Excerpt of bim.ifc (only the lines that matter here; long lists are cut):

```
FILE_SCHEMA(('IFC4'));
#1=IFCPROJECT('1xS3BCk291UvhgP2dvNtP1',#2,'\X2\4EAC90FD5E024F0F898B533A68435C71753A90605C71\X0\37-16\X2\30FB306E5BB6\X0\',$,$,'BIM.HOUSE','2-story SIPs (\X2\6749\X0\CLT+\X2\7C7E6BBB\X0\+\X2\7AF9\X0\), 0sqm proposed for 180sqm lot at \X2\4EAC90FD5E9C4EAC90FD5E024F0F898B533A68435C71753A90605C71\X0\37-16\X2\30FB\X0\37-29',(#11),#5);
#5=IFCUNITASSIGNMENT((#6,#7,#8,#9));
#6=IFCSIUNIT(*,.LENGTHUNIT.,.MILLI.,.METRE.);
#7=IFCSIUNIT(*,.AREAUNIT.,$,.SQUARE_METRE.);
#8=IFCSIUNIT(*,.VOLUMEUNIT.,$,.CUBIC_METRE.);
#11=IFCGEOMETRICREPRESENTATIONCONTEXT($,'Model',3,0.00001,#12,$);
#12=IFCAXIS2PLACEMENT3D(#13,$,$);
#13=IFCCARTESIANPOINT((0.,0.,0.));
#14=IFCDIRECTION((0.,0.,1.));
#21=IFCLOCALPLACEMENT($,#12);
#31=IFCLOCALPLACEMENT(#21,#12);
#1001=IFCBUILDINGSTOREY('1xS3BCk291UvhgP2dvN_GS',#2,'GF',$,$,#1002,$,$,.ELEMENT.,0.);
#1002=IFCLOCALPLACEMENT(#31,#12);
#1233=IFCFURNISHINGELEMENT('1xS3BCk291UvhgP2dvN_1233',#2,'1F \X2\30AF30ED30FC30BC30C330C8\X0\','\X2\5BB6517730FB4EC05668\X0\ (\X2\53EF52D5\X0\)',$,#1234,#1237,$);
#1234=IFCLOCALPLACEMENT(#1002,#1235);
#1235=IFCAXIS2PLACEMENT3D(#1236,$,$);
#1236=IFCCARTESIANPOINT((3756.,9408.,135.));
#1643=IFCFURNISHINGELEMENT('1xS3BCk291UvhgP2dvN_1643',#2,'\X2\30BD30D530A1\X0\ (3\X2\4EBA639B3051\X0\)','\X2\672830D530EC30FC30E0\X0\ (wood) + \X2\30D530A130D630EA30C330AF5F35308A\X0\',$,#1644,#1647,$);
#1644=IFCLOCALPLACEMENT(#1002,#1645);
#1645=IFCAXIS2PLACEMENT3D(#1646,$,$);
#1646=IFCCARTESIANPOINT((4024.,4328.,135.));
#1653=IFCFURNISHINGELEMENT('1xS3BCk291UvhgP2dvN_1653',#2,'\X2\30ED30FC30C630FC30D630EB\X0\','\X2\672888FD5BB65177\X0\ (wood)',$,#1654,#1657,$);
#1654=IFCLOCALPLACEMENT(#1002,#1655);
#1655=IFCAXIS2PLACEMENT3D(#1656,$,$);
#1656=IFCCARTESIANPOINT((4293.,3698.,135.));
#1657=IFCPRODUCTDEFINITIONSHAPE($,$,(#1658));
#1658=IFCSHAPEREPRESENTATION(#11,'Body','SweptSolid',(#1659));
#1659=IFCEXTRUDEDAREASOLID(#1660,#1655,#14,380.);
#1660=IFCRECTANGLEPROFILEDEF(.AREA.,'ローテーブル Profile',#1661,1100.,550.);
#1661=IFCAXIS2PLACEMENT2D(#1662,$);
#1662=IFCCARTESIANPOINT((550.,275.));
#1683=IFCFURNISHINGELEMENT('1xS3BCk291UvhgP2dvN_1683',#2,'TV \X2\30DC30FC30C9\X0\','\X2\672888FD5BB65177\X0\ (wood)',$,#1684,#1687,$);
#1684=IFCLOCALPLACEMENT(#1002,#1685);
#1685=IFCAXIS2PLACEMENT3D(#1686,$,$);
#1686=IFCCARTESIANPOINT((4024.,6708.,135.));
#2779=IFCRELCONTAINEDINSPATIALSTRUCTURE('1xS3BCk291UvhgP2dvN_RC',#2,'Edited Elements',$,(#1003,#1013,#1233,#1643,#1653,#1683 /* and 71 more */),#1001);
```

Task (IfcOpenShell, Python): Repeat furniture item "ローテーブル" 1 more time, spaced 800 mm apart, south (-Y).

```python
import numpy as np
import ifcopenshell
import ifcopenshell.api.geometry
import ifcopenshell.api.root
import ifcopenshell.util.element
import ifcopenshell.util.placement

model = ifcopenshell.open("bim.ifc")


def reuse_history(source, copy):
    """copy_class also copies each property set's owner history, people and application; keep the originals."""
    for rel in copy.IsDefinedBy:
        if rel.is_a("IfcRelDefinesByProperties") and (history := rel.RelatingPropertyDefinition.OwnerHistory):
            rel.RelatingPropertyDefinition.OwnerHistory = source.OwnerHistory
            ifcopenshell.util.element.remove_deep2(model, history)


source = model.by_guid("1xS3BCk291UvhgP2dvN_1653")
base = ifcopenshell.util.placement.get_local_placement(source.ObjectPlacement)
step = np.array([0.0, -1.0, 0.0]) * 800.0

for i in range(1, 2):
    copy = ifcopenshell.api.root.copy_class(model, product=source)
    copy.Representation = ifcopenshell.util.element.copy_deep(
        model, source.Representation, exclude=["IfcGeometricRepresentationContext", "IfcRepresentationMap"]
    )
    reuse_history(source, copy)
    matrix = base.copy()
    matrix[:3, 3] += i * step
    print("added at", matrix[:3, 3].round(3) + 0.0)
    ifcopenshell.api.geometry.edit_object_placement(model, product=copy, matrix=matrix, is_si=False)

model.write("bim_rev.ifc")
```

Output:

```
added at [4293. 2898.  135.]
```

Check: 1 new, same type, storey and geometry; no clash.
